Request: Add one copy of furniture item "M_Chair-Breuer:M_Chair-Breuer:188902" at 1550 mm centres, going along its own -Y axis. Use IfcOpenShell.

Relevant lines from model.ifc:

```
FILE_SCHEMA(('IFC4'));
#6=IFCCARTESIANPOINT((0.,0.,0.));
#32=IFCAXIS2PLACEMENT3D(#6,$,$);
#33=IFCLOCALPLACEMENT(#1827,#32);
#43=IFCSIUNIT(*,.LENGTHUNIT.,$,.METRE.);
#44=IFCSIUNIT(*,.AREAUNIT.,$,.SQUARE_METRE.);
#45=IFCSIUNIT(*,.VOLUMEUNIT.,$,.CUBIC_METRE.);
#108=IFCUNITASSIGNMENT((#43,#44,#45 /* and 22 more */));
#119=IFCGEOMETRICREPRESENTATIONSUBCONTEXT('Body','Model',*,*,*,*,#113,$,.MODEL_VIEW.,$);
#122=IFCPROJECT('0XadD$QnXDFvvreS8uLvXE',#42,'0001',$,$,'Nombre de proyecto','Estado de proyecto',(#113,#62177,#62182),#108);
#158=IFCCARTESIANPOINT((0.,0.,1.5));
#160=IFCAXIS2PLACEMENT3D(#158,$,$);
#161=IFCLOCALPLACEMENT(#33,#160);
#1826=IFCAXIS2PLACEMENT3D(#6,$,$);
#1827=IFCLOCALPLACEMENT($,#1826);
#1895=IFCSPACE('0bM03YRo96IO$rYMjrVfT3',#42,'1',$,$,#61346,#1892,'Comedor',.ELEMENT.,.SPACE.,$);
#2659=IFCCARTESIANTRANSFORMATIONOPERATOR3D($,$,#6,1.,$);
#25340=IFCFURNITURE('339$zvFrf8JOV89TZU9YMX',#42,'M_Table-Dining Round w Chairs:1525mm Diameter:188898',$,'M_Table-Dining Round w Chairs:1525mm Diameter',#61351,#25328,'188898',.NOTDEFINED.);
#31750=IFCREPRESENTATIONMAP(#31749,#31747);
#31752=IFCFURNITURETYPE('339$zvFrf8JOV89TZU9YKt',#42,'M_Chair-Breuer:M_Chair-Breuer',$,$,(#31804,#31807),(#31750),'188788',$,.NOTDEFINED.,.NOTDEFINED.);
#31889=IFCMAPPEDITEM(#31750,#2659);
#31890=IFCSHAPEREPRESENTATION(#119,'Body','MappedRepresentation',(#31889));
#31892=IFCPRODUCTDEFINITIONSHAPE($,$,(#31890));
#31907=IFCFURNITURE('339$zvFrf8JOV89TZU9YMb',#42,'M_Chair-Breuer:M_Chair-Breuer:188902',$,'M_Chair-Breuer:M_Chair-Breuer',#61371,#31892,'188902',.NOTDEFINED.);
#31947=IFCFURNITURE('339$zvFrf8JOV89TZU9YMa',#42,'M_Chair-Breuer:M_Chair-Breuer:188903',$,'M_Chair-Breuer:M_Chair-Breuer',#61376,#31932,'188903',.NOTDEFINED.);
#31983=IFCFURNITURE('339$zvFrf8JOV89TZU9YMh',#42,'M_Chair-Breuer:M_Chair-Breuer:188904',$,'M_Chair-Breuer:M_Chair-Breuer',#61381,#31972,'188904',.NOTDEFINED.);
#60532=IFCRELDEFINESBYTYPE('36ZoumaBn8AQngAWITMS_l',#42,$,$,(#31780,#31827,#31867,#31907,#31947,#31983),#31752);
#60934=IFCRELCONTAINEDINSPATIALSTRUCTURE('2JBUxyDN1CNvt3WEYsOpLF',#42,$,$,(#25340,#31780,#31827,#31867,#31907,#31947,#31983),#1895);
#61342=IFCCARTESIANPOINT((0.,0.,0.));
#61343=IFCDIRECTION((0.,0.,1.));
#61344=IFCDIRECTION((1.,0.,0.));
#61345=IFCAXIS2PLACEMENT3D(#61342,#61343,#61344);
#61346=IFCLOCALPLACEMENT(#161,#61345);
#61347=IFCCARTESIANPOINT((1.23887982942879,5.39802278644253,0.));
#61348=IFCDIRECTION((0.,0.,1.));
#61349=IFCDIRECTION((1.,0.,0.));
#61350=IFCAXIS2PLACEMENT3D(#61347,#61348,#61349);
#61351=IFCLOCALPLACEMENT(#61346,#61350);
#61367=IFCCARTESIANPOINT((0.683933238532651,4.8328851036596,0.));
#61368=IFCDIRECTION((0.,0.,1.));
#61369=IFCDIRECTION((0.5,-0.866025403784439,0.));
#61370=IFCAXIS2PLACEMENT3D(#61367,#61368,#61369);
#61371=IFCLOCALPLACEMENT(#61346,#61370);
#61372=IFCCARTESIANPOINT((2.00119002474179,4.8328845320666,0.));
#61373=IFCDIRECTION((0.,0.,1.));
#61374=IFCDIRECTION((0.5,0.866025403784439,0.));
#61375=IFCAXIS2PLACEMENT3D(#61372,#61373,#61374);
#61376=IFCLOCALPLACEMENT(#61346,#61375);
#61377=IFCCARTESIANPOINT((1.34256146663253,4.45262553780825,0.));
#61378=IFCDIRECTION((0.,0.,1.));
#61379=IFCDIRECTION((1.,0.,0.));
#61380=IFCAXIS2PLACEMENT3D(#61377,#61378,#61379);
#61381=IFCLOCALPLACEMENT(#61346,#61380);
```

```python
import ifcopenshell
import ifcopenshell.api.geometry
import ifcopenshell.api.root
import ifcopenshell.util.element
import ifcopenshell.util.placement
import ifcopenshell.util.unit

model = ifcopenshell.open("model.ifc")
unit_scale = ifcopenshell.util.unit.calculate_unit_scale(model)


def reuse_history(source, copy):
    """copy_class also copies each property set's owner history, people and application; keep the originals."""
    for rel in copy.IsDefinedBy:
        if rel.is_a("IfcRelDefinesByProperties") and (history := rel.RelatingPropertyDefinition.OwnerHistory):
            rel.RelatingPropertyDefinition.OwnerHistory = source.OwnerHistory
            ifcopenshell.util.element.remove_deep2(model, history)


source = model.by_id(31907)
base = ifcopenshell.util.placement.get_local_placement(source.ObjectPlacement)
step = -base[:3, 1] * 1.55 / unit_scale

for i in range(1, 2):
    copy = ifcopenshell.api.root.copy_class(model, product=source)
    copy.Representation = ifcopenshell.util.element.copy_deep(
        model, source.Representation, exclude=["IfcGeometricRepresentationContext", "IfcRepresentationMap"]
    )
    copy.Name = "M_Chair-Breuer:M_Chair-Breuer"
    copy.Tag = None
    reuse_history(source, copy)
    matrix = base.copy()
    matrix[:3, 3] += i * step
    print("added at", matrix[:3, 3].round(3) + 0.0)
    ifcopenshell.api.geometry.edit_object_placement(model, product=copy, matrix=matrix, is_si=False)

model.write("model_edited.ifc")
```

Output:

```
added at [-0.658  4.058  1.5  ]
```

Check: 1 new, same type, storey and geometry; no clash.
